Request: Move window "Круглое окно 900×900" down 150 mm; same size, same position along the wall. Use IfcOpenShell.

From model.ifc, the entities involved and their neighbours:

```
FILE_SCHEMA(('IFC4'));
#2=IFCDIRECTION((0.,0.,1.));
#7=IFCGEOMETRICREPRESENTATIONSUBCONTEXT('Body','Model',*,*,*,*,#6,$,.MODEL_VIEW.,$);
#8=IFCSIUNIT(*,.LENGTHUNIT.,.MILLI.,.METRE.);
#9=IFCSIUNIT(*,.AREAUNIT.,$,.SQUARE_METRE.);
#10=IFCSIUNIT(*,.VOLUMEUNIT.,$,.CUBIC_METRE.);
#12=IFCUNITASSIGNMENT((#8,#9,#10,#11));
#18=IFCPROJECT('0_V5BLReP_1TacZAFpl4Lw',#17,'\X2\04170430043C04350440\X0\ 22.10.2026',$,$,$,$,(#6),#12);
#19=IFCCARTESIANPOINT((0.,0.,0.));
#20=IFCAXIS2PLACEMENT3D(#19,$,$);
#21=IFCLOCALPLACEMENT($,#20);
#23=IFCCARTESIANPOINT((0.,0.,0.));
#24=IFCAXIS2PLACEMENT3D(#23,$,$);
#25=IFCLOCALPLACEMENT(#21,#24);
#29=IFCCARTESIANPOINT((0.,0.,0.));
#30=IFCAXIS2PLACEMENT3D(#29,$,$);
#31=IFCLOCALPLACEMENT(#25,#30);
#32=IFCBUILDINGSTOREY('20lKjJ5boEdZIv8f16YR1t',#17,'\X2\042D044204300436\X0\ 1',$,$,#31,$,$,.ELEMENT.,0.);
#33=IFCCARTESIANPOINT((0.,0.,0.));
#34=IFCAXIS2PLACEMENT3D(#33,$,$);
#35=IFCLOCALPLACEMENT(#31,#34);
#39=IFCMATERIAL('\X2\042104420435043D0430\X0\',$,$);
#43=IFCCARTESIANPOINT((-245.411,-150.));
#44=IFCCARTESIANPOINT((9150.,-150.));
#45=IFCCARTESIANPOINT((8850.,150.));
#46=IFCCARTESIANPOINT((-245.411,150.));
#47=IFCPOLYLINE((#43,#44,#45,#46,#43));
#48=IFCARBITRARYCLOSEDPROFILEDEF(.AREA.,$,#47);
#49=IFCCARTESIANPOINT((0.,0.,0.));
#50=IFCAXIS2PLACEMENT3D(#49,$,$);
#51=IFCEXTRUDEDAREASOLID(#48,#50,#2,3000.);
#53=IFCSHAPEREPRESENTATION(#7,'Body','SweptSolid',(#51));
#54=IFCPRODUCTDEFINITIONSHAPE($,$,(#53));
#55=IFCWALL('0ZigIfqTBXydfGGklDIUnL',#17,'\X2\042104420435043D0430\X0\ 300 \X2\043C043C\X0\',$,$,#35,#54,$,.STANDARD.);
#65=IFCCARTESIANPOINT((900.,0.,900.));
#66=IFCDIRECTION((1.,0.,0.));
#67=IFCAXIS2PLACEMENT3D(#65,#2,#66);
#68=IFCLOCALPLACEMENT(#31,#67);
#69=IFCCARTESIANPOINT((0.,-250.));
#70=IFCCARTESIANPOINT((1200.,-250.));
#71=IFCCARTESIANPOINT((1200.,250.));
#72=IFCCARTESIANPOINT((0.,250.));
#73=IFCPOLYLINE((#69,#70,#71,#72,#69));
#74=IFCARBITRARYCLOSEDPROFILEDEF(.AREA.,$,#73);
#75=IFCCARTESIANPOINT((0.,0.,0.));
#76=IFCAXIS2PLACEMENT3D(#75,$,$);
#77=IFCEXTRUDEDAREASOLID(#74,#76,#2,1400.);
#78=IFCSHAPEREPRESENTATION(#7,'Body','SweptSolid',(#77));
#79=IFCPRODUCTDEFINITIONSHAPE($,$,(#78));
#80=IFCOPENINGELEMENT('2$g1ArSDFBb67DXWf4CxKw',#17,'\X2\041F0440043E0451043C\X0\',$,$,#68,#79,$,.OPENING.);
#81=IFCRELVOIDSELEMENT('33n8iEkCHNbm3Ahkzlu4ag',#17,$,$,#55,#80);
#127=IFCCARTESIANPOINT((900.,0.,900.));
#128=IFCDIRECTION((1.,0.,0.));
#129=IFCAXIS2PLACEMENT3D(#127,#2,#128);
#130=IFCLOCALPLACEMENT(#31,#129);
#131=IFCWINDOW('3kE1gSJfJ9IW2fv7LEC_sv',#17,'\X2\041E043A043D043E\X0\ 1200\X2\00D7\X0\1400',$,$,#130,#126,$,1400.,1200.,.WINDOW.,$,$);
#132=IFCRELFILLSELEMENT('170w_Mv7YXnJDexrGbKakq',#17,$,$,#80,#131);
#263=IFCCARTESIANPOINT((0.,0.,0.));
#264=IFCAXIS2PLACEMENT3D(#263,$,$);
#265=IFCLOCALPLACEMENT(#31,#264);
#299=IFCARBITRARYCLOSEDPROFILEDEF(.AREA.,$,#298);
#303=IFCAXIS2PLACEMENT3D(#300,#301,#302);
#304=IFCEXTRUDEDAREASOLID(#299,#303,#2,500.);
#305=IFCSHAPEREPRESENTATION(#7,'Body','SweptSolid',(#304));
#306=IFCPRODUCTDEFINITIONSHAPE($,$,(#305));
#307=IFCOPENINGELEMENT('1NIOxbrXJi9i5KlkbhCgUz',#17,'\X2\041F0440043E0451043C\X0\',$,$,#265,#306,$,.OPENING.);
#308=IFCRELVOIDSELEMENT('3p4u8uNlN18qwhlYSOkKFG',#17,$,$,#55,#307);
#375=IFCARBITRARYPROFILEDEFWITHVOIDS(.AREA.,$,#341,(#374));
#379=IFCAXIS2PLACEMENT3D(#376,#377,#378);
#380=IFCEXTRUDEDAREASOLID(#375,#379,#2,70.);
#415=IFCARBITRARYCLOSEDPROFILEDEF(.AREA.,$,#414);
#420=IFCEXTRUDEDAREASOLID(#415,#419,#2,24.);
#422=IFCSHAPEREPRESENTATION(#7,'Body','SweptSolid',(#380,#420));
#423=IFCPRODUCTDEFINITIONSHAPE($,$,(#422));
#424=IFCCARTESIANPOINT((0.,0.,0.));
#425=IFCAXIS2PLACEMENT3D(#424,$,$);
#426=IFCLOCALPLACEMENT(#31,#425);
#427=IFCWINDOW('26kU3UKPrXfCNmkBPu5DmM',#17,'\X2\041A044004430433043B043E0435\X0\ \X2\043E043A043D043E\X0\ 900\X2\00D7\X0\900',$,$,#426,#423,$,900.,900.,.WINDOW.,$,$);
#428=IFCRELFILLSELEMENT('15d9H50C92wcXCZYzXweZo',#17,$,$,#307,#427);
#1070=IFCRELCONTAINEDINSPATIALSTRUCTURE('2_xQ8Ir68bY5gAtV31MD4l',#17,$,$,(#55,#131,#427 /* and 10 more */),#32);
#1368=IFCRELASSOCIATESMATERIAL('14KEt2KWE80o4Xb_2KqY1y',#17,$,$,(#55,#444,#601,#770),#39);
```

```python
import numpy as np
import ifcopenshell
import ifcopenshell.api.geometry
import ifcopenshell.util.placement
import ifcopenshell.util.unit

model = ifcopenshell.open("model.ifc")
unit_scale = ifcopenshell.util.unit.calculate_unit_scale(model)

window = model.by_guid("26kU3UKPrXfCNmkBPu5DmM")
opening = window.FillsVoids[0].RelatingOpeningElement
dz = -150.0

shift = np.array([0.0, 0.0, dz])
# The window is not placed relative to its opening, so move both.
for product in (opening, window):
    matrix = ifcopenshell.util.placement.get_local_placement(product.ObjectPlacement)
    matrix[:3, 3] += shift
    ifcopenshell.api.geometry.edit_object_placement(model, product=product, matrix=matrix, is_si=False)

print(f"moved by {dz * unit_scale:+.3f} m")

model.write("model_edited.ifc")
```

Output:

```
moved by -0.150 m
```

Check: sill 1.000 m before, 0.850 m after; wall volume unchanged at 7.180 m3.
